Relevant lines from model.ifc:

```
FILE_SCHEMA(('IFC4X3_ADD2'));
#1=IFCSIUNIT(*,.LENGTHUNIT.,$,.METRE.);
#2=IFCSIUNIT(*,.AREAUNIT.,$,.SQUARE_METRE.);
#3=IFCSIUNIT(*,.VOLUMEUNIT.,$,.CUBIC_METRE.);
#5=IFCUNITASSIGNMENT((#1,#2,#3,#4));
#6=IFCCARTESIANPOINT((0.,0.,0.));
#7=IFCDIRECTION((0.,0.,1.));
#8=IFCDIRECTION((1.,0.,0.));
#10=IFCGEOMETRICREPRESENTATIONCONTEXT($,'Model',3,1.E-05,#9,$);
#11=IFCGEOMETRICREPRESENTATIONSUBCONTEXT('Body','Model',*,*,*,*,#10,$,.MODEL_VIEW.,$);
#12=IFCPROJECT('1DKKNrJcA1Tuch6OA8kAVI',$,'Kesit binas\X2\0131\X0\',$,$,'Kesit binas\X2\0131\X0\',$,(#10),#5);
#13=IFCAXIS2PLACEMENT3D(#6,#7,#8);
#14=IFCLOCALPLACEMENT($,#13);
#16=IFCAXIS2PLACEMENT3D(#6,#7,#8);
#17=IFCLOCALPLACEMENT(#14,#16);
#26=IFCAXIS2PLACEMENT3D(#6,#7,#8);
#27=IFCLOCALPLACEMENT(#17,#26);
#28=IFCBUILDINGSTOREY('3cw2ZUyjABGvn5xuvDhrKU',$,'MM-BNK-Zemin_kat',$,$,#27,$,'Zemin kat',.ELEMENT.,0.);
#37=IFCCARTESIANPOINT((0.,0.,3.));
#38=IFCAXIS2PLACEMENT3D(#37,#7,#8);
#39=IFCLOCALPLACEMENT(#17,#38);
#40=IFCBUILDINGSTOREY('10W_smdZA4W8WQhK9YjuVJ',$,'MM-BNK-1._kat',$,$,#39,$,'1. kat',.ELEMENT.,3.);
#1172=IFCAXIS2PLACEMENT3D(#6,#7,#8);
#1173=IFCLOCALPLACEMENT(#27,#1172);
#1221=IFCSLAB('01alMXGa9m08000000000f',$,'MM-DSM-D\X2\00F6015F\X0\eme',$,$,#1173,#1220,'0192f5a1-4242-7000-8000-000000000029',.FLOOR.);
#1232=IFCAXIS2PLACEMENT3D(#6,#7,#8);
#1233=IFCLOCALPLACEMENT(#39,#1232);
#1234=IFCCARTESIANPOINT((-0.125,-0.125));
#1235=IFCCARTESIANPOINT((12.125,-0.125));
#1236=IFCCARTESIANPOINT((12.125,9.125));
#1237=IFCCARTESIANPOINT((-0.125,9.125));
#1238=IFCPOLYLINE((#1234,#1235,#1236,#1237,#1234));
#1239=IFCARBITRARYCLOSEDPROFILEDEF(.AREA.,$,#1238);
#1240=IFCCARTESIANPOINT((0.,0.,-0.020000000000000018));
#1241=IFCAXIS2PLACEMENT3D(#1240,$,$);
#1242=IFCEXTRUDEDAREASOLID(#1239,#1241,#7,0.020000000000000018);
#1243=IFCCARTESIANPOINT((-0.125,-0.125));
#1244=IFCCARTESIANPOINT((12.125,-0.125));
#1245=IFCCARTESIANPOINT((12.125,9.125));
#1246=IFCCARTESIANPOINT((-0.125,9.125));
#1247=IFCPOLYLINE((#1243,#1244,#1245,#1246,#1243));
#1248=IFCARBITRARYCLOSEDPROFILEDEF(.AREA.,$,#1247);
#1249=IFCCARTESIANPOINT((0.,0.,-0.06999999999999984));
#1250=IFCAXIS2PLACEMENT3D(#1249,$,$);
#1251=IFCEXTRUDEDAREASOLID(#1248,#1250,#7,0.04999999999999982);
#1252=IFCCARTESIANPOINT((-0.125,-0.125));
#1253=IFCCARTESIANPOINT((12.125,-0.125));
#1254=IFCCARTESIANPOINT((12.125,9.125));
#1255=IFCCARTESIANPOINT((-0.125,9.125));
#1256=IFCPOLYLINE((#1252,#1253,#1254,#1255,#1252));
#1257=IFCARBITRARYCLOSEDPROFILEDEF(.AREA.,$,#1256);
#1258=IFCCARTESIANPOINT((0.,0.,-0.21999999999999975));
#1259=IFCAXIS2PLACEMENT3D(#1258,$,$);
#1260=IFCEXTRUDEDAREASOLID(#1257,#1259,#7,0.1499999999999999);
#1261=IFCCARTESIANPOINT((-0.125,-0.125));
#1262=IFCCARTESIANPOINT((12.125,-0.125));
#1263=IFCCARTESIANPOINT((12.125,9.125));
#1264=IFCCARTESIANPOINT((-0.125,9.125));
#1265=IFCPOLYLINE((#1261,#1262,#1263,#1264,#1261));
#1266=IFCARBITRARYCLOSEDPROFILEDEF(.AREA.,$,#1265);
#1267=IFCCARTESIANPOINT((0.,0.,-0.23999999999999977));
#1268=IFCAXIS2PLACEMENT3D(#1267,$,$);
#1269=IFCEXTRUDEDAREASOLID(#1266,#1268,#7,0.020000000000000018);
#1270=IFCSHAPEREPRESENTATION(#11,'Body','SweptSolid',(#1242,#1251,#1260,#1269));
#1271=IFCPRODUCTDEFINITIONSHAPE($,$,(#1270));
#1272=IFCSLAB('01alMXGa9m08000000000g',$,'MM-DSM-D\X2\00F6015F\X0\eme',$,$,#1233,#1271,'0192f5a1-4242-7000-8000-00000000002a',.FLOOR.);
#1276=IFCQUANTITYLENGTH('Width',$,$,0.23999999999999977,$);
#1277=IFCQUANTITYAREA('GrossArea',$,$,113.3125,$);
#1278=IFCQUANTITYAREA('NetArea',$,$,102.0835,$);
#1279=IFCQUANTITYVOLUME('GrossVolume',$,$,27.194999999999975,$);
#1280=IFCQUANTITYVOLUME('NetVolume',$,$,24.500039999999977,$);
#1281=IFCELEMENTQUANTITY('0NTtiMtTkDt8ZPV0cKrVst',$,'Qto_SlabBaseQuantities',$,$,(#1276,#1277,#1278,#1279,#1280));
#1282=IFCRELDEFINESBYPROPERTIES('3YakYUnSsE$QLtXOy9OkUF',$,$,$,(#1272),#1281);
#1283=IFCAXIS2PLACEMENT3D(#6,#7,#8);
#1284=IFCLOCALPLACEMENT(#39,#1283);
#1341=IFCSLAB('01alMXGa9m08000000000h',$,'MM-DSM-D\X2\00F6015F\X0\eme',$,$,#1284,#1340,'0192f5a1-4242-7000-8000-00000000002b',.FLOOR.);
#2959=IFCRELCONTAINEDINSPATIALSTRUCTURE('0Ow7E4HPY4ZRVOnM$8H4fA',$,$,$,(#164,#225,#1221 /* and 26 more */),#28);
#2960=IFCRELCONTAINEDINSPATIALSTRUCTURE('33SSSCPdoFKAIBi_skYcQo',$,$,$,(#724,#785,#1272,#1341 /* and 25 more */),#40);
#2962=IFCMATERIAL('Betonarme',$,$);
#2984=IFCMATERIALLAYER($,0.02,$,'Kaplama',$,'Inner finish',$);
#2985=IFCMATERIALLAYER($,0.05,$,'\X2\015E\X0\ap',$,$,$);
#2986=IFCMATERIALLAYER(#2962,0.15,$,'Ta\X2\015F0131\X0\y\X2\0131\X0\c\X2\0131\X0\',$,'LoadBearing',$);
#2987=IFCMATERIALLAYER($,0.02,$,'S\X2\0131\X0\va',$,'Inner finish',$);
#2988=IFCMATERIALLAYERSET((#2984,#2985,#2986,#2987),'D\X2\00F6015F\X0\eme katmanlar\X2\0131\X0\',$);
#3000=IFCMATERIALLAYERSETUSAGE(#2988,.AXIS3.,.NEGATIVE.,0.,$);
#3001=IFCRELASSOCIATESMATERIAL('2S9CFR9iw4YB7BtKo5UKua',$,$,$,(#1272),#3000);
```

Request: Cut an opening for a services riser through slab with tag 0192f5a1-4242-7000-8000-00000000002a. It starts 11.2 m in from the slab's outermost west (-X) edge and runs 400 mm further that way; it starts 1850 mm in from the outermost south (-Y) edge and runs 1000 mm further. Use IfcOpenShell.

```python
import numpy as np
import ifcopenshell
import ifcopenshell.api.feature
import ifcopenshell.api.geometry
import ifcopenshell.api.pset
import ifcopenshell.api.root
import ifcopenshell.geom
import ifcopenshell.util.element
import ifcopenshell.util.placement
import ifcopenshell.util.representation
import ifcopenshell.util.shape
import ifcopenshell.util.unit

model = ifcopenshell.open("model.ifc")
unit_scale = ifcopenshell.util.unit.calculate_unit_scale(model)
area_scale = ifcopenshell.util.unit.calculate_unit_scale(model, "AREAUNIT")
volume_scale = ifcopenshell.util.unit.calculate_unit_scale(model, "VOLUMEUNIT")
settings = ifcopenshell.geom.settings()


def volume(element):
    """Net volume in cubic metres, openings subtracted."""
    shape = ifcopenshell.geom.create_shape(settings, element)
    return ifcopenshell.util.shape.get_volume(shape.geometry)


slab = model.by_guid("01alMXGa9m08000000000g")
before = volume(slab)

# Extent in the slab's own axes, in metres. The edges named are its -X and -Y sides.
slab_shape = ifcopenshell.geom.create_shape(settings, slab)
vertices = ifcopenshell.util.shape.get_vertices(slab_shape.geometry)
x_min, y_min, bottom = vertices.min(axis=0)
top = vertices[:, 2].max()

opening = ifcopenshell.api.root.create_entity(model, ifc_class="IfcOpeningElement", name="Services riser opening", predefined_type="OPENING")
context = ifcopenshell.util.representation.get_context(model, "Model", "Body", "MODEL_VIEW")
width, depth = 0.4, 1
outline = [(0.0, 0.0), (width, 0.0), (width, depth), (0.0, depth), (0.0, 0.0)]
# Overshoot both faces by 50 mm so the cut is clean.
shape = ifcopenshell.api.geometry.add_slab_representation(
    model, context=context, depth=top - bottom + 0.1, polyline=outline
)
ifcopenshell.api.geometry.assign_representation(model, product=opening, representation=shape)

matrix = ifcopenshell.util.placement.get_local_placement(slab.ObjectPlacement)
matrix[:, 3] = matrix @ np.append(np.array([x_min + 11.2, y_min + 1.85, bottom - 0.05]) / unit_scale, 1.0)
ifcopenshell.api.geometry.edit_object_placement(model, product=opening, matrix=matrix, is_si=False)
ifcopenshell.api.feature.add_feature(model, feature=opening, element=slab)

after = volume(slab)

# Update the slab's stored quantities.
qto = model.by_id(ifcopenshell.util.element.get_pset(slab, "Qto_SlabBaseQuantities", should_inherit=False)["id"])
ifcopenshell.api.pset.edit_qto(model, qto=qto, properties={
    "NetArea": after / (top - bottom) / area_scale,
    "NetVolume": after / volume_scale,
})

print(f"slab volume {before:.3f} -> {after:.3f} m3")

model.write("model_rev.ifc")
```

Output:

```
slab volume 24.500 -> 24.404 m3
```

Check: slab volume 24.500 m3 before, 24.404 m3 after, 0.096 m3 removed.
